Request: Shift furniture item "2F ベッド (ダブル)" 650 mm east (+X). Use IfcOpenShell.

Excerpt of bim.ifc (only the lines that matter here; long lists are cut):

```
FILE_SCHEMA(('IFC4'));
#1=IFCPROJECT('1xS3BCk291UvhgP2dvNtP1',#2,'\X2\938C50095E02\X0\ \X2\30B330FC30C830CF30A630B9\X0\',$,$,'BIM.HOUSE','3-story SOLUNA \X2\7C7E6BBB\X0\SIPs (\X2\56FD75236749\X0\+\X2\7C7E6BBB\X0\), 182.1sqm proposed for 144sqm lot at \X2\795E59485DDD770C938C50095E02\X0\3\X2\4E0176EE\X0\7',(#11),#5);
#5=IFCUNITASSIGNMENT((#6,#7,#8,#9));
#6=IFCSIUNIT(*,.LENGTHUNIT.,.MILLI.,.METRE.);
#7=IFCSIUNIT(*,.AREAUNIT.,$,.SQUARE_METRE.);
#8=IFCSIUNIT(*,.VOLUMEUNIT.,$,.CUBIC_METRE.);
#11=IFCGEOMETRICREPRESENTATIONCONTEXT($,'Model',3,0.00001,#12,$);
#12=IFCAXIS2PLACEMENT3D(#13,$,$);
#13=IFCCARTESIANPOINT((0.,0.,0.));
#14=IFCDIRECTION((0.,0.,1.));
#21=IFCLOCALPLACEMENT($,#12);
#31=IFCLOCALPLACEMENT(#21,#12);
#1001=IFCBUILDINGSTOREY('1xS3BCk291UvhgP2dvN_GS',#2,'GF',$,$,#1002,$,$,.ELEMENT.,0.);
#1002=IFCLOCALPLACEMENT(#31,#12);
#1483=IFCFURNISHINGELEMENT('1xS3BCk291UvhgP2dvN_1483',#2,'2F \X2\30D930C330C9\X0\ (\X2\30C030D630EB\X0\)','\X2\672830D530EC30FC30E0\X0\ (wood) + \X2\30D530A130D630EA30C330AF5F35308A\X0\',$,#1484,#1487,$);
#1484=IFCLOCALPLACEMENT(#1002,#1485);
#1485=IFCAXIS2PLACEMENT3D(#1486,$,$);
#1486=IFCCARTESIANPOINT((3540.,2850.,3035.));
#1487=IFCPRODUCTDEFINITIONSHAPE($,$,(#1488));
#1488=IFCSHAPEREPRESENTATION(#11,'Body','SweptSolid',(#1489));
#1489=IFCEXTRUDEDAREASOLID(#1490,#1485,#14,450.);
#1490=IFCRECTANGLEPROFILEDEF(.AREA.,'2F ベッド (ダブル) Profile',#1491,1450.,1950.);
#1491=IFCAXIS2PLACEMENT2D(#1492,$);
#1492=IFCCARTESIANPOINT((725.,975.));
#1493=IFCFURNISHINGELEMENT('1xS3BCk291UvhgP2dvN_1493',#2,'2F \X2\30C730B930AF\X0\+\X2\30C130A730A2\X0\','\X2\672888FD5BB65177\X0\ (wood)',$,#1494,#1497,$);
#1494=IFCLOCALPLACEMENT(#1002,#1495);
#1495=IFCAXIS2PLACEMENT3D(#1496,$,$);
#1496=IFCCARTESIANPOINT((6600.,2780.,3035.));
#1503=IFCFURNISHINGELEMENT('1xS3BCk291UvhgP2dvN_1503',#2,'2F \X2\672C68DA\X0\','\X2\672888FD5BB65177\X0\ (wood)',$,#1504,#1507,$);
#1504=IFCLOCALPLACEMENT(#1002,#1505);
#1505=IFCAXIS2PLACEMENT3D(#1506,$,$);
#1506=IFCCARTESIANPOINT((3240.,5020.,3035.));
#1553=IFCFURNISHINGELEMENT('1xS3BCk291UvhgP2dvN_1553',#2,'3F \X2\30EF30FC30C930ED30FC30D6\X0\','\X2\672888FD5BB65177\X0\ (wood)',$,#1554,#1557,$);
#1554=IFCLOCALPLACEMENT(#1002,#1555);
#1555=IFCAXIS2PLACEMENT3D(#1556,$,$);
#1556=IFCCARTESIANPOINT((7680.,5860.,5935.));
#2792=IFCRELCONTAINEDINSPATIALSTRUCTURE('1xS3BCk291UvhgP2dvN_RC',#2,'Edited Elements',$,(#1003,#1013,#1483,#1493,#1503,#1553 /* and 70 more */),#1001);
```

```python
import ifcopenshell
import ifcopenshell.api.geometry
import ifcopenshell.util.placement
import ifcopenshell.util.unit

model = ifcopenshell.open("bim.ifc")
unit_scale = ifcopenshell.util.unit.calculate_unit_scale(model)

item = model.by_guid("1xS3BCk291UvhgP2dvN_1483")
matrix = ifcopenshell.util.placement.get_local_placement(item.ObjectPlacement)
matrix[0, 3] += 0.65 / unit_scale
ifcopenshell.api.geometry.edit_object_placement(model, product=item, matrix=matrix, is_si=False)

print(ifcopenshell.util.placement.get_local_placement(item.ObjectPlacement).round(3) + 0.0)

model.write("bim_updated.ifc")
```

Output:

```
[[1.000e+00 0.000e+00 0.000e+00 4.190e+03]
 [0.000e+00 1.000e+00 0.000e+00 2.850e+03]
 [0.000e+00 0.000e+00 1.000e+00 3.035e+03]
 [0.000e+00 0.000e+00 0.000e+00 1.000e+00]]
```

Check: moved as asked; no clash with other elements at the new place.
